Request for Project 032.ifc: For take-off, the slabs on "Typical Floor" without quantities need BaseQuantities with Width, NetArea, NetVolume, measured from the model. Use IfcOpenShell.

First a look at what the model holds.

```python
import ifcopenshell
import ifcopenshell.util.element
import ifcopenshell.util.unit

model = ifcopenshell.open("Project 032.ifc")
print(model.schema)
for unit_type in ("LENGTHUNIT", "AREAUNIT", "VOLUMEUNIT"):
    print(unit_type, ifcopenshell.util.unit.calculate_unit_scale(model, unit_type))
storey = next(s for s in model.by_type("IfcBuildingStorey") if s.Name == "Typical Floor")
slabs = [e for e in ifcopenshell.util.element.get_decomposition(storey) if e.is_a("IfcSlab")]
for e in sorted(slabs, key=lambda e: e.id()):
    print(e.id(), e.is_a(), e.Name, list(ifcopenshell.util.element.get_psets(e, qtos_only=True)), sep=" | ")
```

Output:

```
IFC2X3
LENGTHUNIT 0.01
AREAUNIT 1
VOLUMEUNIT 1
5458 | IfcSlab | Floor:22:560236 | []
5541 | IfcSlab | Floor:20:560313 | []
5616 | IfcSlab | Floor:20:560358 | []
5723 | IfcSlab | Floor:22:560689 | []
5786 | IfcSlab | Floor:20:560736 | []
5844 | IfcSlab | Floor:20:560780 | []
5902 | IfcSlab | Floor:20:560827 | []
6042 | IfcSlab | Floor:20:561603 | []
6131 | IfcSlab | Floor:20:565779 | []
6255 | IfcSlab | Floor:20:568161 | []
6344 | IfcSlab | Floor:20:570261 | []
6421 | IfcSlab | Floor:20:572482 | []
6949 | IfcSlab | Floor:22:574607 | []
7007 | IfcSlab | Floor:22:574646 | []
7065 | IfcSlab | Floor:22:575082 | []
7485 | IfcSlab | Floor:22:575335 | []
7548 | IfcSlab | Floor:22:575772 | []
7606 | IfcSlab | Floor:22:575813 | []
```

```python
import ifcopenshell
import ifcopenshell.api.pset
import ifcopenshell.geom
import ifcopenshell.util.element
import ifcopenshell.util.shape
import ifcopenshell.util.unit

model = ifcopenshell.open("Project 032.ifc")
unit_scale = ifcopenshell.util.unit.calculate_unit_scale(model)
area_scale = ifcopenshell.util.unit.calculate_unit_scale(model, "AREAUNIT")
volume_scale = ifcopenshell.util.unit.calculate_unit_scale(model, "VOLUMEUNIT")
settings = ifcopenshell.geom.settings()

storey = next(s for s in model.by_type("IfcBuildingStorey") if s.Name == "Typical Floor")
slabs = [e for e in ifcopenshell.util.element.get_decomposition(storey) if e.is_a("IfcSlab")]

for e in sorted(slabs, key=lambda e: e.id()):
    if ifcopenshell.util.element.get_psets(e, qtos_only=True, should_inherit=False):
        continue
    # Geometry comes back in metres, in the element's own axes.
    shape = ifcopenshell.geom.create_shape(settings, e)
    values = {
        "Width": ifcopenshell.util.shape.get_z(shape.geometry) / unit_scale,
        "NetArea": ifcopenshell.util.shape.get_footprint_area(shape.geometry) / area_scale,
        "NetVolume": ifcopenshell.util.shape.get_volume(shape.geometry) / volume_scale,
    }
    qto = ifcopenshell.api.pset.add_qto(model, product=e, name="BaseQuantities")
    ifcopenshell.api.pset.edit_qto(model, qto=qto, properties=values)
    print(e.id(), {k: round(v, 3) for k, v in values.items()})

model.write("Project 032_rev.ifc")
```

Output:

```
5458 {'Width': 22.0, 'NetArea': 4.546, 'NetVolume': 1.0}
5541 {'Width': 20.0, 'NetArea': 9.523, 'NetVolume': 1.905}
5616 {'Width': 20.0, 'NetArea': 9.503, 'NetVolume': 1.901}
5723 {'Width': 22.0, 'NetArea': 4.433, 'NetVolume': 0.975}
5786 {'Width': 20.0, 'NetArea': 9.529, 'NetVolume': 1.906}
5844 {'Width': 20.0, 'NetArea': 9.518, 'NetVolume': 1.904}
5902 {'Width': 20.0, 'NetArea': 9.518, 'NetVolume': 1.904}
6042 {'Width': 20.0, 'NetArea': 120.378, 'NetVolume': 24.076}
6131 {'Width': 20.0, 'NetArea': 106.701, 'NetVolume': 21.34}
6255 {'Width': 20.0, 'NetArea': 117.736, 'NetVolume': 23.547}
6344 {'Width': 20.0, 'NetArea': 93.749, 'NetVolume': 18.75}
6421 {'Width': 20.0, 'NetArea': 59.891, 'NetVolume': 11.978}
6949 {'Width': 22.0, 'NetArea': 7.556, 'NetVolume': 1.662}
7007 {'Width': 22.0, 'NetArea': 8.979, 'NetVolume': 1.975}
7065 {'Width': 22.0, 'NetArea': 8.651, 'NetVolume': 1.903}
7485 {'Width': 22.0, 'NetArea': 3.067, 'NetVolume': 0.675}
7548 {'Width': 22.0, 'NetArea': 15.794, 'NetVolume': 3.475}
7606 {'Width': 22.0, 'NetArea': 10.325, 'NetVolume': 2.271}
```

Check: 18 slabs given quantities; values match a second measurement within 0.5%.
